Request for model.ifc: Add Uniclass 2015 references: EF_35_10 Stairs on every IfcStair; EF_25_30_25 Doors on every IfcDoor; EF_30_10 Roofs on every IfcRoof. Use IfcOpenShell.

First a look at what the model holds.

```python
import ifcopenshell

model = ifcopenshell.open("model.ifc")
print(model.schema)
print("classifications:", [c.Name for c in model.by_type("IfcClassification")])
for ifc_class in ("IfcDoor", "IfcRoof", "IfcStair", "IfcWall", "IfcWindow"):
    print(ifc_class, len(model.by_type(ifc_class)))
```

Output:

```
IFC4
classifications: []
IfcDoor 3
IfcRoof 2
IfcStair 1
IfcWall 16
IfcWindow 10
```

```python
import ifcopenshell
import ifcopenshell.api.classification

model = ifcopenshell.open("model.ifc")

system = ifcopenshell.api.classification.add_classification(model, classification="Uniclass 2015")

codes = {
    "IfcStair": ("EF_35_10", "Stairs"),
    "IfcDoor": ("EF_25_30_25", "Doors"),
    "IfcRoof": ("EF_30_10", "Roofs"),
}
for ifc_class, (code, name) in codes.items():
    products = model.by_type(ifc_class)
    ifcopenshell.api.classification.add_reference(
        model, products=products, classification=system, identification=code, name=name
    )
    print(code, len(products))

model.write("model-out.ifc")
```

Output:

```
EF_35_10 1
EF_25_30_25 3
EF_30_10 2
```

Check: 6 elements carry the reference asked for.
